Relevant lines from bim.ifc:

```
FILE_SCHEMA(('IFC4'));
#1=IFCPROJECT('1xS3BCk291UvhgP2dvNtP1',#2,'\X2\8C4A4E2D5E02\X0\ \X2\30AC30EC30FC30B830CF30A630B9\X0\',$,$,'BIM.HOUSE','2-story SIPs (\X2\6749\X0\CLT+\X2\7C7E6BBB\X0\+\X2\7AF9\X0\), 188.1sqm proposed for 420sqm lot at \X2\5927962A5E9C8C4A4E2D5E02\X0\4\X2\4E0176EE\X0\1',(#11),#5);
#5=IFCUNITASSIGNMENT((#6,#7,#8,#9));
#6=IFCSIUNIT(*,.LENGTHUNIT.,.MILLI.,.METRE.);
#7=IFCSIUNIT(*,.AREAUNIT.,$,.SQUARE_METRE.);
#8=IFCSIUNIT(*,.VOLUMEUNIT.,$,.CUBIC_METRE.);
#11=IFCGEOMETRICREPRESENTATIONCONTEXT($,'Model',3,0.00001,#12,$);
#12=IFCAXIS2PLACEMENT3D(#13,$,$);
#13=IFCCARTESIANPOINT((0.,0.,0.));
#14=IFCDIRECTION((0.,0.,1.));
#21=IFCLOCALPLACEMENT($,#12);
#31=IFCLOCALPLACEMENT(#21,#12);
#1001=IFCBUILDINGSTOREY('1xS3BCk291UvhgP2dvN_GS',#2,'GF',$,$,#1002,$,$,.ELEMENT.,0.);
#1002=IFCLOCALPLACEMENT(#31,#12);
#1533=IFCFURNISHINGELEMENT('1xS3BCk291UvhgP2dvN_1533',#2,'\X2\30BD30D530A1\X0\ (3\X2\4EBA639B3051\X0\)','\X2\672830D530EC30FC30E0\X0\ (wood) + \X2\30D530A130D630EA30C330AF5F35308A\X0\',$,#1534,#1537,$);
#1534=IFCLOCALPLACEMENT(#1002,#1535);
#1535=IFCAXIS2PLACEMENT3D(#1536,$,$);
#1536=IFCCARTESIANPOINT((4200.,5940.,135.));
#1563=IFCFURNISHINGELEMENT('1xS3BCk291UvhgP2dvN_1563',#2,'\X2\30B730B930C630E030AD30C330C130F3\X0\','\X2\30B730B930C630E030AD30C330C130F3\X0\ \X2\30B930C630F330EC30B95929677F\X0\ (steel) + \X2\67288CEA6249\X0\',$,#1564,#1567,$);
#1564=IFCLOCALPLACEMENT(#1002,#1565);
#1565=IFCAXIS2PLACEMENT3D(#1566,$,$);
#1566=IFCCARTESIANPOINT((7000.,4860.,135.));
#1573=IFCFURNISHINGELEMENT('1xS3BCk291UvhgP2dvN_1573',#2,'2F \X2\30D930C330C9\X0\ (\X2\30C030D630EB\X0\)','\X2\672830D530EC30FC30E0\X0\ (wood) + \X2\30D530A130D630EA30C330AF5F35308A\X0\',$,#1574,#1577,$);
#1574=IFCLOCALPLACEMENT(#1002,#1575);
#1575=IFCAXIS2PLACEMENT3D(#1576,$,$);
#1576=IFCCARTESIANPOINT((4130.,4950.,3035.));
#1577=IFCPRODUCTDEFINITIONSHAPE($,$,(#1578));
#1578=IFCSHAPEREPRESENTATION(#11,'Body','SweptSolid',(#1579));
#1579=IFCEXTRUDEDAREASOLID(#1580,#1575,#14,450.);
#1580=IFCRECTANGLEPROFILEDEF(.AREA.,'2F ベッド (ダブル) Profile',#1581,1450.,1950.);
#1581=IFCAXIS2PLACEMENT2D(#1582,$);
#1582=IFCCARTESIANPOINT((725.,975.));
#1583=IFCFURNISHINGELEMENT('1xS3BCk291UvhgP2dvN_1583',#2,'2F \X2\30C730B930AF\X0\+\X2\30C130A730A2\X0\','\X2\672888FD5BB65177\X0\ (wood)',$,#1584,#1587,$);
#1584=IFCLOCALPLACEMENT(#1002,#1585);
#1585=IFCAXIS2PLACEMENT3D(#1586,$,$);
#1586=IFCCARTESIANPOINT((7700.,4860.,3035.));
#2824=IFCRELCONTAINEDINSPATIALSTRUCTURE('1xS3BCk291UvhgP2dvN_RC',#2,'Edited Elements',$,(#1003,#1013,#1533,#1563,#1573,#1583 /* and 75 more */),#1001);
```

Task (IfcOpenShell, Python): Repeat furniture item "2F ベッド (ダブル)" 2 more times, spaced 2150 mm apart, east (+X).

```python
import numpy as np
import ifcopenshell
import ifcopenshell.api.geometry
import ifcopenshell.api.root
import ifcopenshell.util.element
import ifcopenshell.util.placement

model = ifcopenshell.open("bim.ifc")


def reuse_history(source, copy):
    """copy_class also copies each property set's owner history, people and application; keep the originals."""
    for rel in copy.IsDefinedBy:
        if rel.is_a("IfcRelDefinesByProperties") and (history := rel.RelatingPropertyDefinition.OwnerHistory):
            rel.RelatingPropertyDefinition.OwnerHistory = source.OwnerHistory
            ifcopenshell.util.element.remove_deep2(model, history)


source = model.by_guid("1xS3BCk291UvhgP2dvN_1573")
base = ifcopenshell.util.placement.get_local_placement(source.ObjectPlacement)
step = np.array([1.0, 0.0, 0.0]) * 2150.0

for i in range(1, 3):
    copy = ifcopenshell.api.root.copy_class(model, product=source)
    copy.Representation = ifcopenshell.util.element.copy_deep(
        model, source.Representation, exclude=["IfcGeometricRepresentationContext", "IfcRepresentationMap"]
    )
    reuse_history(source, copy)
    matrix = base.copy()
    matrix[:3, 3] += i * step
    print("added at", matrix[:3, 3].round(3) + 0.0)
    ifcopenshell.api.geometry.edit_object_placement(model, product=copy, matrix=matrix, is_si=False)

model.write("bim_v2.ifc")
```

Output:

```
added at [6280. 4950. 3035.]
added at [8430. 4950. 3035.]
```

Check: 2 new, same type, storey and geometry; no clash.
